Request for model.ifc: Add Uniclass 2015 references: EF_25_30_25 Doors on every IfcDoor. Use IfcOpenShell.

First a look at what the model holds.

```python
import ifcopenshell

model = ifcopenshell.open("model.ifc")
print(model.schema)
print("classifications:", [c.Name for c in model.by_type("IfcClassification")])
for ifc_class in ("IfcDoor", "IfcRoof", "IfcStair", "IfcWall", "IfcWindow"):
    print(ifc_class, len(model.by_type(ifc_class)))
```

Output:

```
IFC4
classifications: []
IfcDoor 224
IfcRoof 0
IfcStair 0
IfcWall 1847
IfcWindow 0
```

```python
import ifcopenshell
import ifcopenshell.api.classification

model = ifcopenshell.open("model.ifc")

system = ifcopenshell.api.classification.add_classification(model, classification="Uniclass 2015")

codes = {
    "IfcDoor": ("EF_25_30_25", "Doors"),
}
for ifc_class, (code, name) in codes.items():
    products = model.by_type(ifc_class)
    ifcopenshell.api.classification.add_reference(
        model, products=products, classification=system, identification=code, name=name
    )
    print(code, len(products))

model.write("model_rev.ifc")
```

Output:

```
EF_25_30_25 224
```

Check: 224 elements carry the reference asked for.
